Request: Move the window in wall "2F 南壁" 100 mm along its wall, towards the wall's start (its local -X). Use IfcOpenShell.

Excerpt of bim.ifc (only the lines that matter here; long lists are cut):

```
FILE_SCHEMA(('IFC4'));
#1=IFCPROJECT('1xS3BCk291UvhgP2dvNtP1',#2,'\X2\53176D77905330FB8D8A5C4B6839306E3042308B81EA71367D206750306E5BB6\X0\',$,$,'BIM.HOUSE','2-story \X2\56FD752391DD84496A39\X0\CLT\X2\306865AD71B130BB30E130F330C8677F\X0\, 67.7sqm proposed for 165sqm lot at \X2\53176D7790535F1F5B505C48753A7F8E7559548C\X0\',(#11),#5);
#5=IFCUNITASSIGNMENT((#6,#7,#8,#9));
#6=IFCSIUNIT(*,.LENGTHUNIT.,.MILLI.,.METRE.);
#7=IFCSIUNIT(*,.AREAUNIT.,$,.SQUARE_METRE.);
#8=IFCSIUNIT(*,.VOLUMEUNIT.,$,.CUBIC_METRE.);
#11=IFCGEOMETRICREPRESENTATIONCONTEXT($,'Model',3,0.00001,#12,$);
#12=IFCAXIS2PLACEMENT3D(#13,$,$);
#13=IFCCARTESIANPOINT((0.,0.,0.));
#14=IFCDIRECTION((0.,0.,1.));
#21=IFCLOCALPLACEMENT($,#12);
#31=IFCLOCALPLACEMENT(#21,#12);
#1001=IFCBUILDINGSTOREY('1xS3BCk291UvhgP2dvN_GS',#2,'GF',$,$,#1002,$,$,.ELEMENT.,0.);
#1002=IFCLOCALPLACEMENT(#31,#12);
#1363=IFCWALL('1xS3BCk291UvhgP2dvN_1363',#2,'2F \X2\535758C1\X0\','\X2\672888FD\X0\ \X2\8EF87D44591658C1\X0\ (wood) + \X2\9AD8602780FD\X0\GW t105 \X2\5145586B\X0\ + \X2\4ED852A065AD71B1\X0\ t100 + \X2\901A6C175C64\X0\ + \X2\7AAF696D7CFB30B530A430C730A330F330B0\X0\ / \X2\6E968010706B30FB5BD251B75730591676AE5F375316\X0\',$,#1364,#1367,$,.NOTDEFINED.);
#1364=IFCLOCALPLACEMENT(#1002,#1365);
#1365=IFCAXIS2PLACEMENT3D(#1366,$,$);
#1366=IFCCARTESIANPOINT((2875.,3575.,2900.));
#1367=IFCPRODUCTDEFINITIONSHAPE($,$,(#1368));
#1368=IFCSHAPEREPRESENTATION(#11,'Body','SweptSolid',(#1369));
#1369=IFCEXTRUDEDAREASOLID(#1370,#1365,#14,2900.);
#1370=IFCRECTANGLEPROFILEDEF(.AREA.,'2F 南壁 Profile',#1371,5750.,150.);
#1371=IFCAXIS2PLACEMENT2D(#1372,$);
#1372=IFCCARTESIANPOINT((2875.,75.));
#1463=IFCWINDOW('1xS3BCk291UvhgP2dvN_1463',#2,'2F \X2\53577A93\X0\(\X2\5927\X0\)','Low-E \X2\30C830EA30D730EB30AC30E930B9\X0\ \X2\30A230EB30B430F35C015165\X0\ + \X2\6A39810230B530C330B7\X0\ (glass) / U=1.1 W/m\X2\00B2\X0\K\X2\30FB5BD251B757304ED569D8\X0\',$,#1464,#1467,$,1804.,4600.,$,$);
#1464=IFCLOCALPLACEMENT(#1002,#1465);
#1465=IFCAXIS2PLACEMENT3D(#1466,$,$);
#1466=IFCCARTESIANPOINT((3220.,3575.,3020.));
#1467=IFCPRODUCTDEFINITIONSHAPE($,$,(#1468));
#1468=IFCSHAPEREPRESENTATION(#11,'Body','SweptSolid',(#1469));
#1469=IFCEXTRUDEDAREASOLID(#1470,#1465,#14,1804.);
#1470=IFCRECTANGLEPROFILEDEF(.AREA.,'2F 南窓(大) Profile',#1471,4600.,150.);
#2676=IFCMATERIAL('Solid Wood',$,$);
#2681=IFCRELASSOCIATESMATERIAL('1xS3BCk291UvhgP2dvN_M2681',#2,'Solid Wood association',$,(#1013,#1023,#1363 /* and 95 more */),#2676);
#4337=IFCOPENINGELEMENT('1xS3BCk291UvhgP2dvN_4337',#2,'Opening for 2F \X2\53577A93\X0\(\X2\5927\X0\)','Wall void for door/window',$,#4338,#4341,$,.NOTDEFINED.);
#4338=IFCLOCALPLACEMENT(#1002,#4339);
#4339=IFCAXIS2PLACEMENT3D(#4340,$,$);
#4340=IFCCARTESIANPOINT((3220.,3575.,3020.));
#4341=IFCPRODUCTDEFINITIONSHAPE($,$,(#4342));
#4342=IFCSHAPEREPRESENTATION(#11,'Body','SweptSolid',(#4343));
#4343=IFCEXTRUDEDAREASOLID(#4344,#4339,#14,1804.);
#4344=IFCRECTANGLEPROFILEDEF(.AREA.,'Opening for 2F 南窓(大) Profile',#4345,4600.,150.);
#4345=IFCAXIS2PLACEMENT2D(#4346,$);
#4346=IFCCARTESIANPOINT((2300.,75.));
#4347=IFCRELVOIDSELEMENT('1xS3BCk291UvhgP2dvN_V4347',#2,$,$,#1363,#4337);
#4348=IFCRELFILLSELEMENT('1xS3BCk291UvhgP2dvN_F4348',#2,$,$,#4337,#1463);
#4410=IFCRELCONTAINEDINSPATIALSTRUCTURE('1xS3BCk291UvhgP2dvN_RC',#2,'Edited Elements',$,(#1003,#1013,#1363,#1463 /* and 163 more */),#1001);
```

```python
import ifcopenshell
import ifcopenshell.api.geometry
import ifcopenshell.util.placement

model = ifcopenshell.open("bim.ifc")

window = model.by_guid("1xS3BCk291UvhgP2dvN_1463")
opening = window.FillsVoids[0].RelatingOpeningElement
wall = opening.VoidsElements[0].RelatingBuildingElement

wall_matrix = ifcopenshell.util.placement.get_local_placement(wall.ObjectPlacement)
shift = wall_matrix[:3, 0] * -100.0
before = ifcopenshell.util.placement.get_local_placement(window.ObjectPlacement)[:3, 3].copy()

# The window is not placed relative to its opening, so move both.
for product in (opening, window):
    matrix = ifcopenshell.util.placement.get_local_placement(product.ObjectPlacement)
    matrix[:3, 3] += shift
    ifcopenshell.api.geometry.edit_object_placement(model, product=product, matrix=matrix, is_si=False)

after = ifcopenshell.util.placement.get_local_placement(window.ObjectPlacement)[:3, 3]
print("window moved by", (after - before).round(3) + 0.0)

model.write("bim_rev.ifc")
```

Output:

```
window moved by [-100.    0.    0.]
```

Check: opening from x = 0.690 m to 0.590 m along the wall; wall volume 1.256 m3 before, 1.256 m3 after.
